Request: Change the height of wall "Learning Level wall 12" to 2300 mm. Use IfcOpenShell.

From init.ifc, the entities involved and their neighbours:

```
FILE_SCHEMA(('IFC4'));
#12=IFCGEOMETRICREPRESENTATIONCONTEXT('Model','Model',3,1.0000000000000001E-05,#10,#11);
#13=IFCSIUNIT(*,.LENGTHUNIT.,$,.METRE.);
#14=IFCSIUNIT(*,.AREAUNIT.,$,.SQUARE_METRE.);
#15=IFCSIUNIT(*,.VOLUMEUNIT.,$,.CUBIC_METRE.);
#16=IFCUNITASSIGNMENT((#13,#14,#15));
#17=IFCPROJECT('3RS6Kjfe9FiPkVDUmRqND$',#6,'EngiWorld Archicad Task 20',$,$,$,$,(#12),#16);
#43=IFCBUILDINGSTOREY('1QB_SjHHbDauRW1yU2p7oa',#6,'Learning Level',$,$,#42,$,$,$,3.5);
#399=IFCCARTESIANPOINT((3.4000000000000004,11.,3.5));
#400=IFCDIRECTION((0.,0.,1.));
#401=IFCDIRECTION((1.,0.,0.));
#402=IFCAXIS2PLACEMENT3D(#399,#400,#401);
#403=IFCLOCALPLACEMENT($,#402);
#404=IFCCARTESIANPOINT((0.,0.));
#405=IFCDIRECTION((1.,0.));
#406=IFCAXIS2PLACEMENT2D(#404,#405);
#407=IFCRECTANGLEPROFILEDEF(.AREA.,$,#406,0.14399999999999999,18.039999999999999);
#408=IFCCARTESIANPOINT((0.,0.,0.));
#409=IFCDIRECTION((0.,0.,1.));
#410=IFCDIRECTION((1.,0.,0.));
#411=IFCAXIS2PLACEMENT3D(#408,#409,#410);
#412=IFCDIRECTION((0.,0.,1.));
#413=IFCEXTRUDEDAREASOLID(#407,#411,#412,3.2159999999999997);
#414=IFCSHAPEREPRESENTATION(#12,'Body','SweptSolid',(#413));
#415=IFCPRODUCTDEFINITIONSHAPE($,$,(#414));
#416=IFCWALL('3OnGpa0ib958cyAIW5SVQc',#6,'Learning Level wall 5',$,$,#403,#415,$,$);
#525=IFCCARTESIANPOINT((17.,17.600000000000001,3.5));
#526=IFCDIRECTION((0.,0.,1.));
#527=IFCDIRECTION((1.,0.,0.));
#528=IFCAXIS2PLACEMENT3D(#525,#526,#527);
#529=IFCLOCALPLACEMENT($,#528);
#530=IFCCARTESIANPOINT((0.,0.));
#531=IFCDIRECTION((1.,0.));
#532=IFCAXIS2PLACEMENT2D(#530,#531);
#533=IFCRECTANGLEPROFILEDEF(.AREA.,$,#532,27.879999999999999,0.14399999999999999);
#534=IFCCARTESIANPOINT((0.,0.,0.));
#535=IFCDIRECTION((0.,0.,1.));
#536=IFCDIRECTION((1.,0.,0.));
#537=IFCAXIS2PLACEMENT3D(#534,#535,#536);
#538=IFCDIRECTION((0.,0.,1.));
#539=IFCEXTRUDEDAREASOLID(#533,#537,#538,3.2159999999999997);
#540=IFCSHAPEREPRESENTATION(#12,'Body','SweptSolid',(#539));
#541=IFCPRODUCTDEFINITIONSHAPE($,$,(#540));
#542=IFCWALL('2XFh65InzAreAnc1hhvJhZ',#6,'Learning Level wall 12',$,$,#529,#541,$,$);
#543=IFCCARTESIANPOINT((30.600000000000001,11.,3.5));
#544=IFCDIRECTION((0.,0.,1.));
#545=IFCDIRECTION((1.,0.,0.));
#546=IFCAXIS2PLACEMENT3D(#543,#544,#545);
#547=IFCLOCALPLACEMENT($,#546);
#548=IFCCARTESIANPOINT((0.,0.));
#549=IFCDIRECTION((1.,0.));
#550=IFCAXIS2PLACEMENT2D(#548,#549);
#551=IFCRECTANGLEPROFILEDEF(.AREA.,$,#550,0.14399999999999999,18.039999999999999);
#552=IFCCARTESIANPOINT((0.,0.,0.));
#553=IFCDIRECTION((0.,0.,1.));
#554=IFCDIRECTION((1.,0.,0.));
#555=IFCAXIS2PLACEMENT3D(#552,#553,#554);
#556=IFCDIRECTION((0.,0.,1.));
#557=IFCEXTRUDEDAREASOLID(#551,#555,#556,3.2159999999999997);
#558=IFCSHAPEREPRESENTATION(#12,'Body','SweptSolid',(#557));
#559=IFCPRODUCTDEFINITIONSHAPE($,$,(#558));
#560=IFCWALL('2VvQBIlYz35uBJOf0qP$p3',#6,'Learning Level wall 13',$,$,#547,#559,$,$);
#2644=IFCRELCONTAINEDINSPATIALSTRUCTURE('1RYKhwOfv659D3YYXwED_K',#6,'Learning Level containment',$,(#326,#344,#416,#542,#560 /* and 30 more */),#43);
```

```python
import ifcopenshell
import ifcopenshell.geom
import ifcopenshell.util.shape
import ifcopenshell.util.unit

model = ifcopenshell.open("init.ifc")
unit_scale = ifcopenshell.util.unit.calculate_unit_scale(model)
settings = ifcopenshell.geom.settings()


def volume(element):
    """Net volume in cubic metres, openings subtracted."""
    shape = ifcopenshell.geom.create_shape(settings, element)
    return ifcopenshell.util.shape.get_volume(shape.geometry)


wall = model.by_guid("2XFh65InzAreAnc1hhvJhZ")
before = volume(wall)

body = next(r for r in wall.Representation.Representations if r.RepresentationIdentifier == "Body")
solid = body.Items[0]
old_height = solid.Depth
solid.Depth = 2.3 / unit_scale
after = volume(wall)

print(f"height {old_height:g} -> {solid.Depth:g}, volume {before:.3f} -> {after:.3f} m3")

model.write("init-out.ifc")
```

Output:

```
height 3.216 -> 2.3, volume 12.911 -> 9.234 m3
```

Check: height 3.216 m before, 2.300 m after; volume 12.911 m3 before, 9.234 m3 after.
